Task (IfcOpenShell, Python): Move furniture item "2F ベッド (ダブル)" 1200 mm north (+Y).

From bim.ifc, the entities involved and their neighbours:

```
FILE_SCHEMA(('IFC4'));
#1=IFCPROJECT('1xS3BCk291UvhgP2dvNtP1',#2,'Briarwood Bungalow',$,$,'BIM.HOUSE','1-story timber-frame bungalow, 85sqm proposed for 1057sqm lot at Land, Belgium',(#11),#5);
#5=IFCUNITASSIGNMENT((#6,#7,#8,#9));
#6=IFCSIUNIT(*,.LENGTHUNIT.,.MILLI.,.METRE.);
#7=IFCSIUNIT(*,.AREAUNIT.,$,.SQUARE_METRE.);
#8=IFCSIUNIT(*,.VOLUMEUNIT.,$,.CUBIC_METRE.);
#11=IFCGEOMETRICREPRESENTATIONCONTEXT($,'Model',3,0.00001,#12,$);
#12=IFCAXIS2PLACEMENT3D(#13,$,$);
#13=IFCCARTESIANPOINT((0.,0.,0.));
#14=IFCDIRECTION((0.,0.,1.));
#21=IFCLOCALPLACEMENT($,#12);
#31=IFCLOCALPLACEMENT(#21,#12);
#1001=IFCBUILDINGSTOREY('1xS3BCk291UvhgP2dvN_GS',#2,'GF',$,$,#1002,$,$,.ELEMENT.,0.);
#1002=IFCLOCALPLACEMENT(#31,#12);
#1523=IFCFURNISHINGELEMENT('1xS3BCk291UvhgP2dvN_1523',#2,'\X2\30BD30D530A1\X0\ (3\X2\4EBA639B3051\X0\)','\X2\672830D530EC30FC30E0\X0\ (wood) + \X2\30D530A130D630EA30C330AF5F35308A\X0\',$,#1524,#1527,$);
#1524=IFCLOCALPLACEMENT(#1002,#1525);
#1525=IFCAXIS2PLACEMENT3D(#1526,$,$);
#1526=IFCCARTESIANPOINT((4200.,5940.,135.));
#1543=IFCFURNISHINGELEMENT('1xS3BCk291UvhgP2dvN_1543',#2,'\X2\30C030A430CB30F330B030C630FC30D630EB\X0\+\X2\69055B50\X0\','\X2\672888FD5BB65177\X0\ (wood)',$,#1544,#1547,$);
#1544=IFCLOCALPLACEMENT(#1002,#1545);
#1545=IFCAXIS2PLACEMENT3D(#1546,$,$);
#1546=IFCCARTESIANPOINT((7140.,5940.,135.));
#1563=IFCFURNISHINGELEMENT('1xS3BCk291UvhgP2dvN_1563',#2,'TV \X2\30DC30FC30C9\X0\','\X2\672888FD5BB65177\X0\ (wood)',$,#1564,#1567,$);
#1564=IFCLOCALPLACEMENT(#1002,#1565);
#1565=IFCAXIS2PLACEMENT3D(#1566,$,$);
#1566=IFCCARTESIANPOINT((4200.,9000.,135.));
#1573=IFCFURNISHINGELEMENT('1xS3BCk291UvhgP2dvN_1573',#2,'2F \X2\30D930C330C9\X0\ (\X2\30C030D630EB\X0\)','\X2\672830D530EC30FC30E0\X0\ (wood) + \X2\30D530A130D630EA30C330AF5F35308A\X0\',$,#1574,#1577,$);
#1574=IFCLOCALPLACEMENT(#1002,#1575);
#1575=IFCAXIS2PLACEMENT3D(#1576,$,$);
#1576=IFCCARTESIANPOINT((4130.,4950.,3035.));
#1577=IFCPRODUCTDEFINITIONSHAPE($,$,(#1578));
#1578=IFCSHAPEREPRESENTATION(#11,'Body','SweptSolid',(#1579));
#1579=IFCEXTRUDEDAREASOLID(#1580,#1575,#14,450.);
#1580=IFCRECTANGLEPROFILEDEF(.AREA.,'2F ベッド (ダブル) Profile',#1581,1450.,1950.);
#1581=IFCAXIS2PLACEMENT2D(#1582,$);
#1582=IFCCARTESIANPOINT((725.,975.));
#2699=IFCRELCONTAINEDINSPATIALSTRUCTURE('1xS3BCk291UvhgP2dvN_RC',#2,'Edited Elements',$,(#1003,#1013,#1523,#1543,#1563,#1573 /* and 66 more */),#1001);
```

```python
import ifcopenshell
import ifcopenshell.api.geometry
import ifcopenshell.util.placement
import ifcopenshell.util.unit

model = ifcopenshell.open("bim.ifc")
unit_scale = ifcopenshell.util.unit.calculate_unit_scale(model)

item = model.by_id(1573)
matrix = ifcopenshell.util.placement.get_local_placement(item.ObjectPlacement)
matrix[1, 3] += 1.2 / unit_scale
ifcopenshell.api.geometry.edit_object_placement(model, product=item, matrix=matrix, is_si=False)

print(ifcopenshell.util.placement.get_local_placement(item.ObjectPlacement).round(3) + 0.0)

model.write("bim-out.ifc")
```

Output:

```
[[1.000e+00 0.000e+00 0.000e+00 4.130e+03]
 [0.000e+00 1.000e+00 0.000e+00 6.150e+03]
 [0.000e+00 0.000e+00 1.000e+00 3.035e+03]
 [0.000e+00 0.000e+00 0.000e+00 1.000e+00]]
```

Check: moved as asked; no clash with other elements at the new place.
